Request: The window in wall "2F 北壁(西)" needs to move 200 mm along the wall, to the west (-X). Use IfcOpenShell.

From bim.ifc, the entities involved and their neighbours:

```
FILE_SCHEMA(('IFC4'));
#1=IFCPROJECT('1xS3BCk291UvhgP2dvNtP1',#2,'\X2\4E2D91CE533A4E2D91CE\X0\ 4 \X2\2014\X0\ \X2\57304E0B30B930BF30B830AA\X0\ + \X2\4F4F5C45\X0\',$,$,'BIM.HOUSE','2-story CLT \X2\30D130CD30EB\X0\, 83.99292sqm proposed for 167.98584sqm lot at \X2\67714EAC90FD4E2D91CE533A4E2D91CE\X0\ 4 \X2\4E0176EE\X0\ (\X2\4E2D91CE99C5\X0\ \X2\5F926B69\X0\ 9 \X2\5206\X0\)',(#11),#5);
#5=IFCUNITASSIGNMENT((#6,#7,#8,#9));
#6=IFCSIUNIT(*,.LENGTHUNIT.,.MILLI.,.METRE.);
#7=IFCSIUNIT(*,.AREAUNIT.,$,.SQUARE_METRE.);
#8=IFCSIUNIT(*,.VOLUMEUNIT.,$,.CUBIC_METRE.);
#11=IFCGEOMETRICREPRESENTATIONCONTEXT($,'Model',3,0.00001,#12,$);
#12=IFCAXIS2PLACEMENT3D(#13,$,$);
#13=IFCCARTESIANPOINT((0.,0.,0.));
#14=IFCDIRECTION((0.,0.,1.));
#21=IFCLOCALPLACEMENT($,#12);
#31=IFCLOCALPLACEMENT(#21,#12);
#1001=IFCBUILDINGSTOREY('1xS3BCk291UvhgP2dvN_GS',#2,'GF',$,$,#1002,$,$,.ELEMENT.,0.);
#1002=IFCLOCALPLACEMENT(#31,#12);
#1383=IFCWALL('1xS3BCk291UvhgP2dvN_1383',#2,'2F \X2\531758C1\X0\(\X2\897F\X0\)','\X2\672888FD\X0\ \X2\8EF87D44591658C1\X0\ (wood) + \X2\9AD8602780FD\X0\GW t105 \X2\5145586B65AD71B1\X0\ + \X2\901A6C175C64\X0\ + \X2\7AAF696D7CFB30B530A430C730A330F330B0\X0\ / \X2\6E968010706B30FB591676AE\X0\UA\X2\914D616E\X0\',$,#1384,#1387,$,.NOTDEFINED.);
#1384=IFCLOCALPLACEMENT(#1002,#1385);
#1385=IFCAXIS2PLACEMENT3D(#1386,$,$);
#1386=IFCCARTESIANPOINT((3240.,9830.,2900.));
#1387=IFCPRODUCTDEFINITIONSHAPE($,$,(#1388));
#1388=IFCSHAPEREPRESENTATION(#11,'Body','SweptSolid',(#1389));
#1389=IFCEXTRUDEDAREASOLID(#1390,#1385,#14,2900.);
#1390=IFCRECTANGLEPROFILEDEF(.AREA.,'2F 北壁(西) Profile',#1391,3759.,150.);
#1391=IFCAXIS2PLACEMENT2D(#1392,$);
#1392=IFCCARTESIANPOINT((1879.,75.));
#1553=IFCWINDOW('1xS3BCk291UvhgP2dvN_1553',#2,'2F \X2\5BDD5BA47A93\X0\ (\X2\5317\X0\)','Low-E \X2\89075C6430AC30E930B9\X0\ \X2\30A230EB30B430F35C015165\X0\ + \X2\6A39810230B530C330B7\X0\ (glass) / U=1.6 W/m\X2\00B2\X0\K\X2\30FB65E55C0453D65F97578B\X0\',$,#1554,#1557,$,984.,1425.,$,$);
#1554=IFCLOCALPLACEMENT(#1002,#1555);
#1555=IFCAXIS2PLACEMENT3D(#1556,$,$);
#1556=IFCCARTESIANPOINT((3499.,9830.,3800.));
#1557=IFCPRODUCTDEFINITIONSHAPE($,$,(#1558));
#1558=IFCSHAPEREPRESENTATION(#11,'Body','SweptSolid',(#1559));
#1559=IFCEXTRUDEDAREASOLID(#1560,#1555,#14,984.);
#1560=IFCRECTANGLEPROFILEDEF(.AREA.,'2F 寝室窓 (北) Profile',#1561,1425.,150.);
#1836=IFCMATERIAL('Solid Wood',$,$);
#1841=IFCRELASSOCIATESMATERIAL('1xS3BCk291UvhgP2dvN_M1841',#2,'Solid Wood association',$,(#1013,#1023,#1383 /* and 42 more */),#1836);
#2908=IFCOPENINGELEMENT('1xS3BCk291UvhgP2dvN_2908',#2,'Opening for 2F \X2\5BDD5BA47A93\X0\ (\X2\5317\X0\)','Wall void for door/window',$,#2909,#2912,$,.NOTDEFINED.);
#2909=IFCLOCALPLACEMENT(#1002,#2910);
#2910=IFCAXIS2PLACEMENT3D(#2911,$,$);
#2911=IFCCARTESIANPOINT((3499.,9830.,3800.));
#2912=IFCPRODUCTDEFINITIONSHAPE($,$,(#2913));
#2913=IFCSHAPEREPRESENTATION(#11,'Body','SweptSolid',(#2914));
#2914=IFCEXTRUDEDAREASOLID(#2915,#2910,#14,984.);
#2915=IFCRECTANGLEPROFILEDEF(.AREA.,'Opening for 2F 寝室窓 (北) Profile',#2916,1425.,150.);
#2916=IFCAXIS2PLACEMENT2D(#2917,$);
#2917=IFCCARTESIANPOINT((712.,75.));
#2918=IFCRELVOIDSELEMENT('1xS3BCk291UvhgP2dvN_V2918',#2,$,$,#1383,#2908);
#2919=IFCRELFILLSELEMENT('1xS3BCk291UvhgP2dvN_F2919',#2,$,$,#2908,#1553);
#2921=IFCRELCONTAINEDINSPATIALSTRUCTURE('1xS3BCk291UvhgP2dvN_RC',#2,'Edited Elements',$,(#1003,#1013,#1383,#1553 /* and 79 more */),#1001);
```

```python
import ifcopenshell
import ifcopenshell.api.geometry
import ifcopenshell.util.placement
import ifcopenshell.util.unit

model = ifcopenshell.open("bim.ifc")
unit_scale = ifcopenshell.util.unit.calculate_unit_scale(model)

window = model.by_guid("1xS3BCk291UvhgP2dvN_1553")
opening = window.FillsVoids[0].RelatingOpeningElement
wall = opening.VoidsElements[0].RelatingBuildingElement

wall_matrix = ifcopenshell.util.placement.get_local_placement(wall.ObjectPlacement)
shift = wall_matrix[:3, 0] * -0.2 / unit_scale
before = ifcopenshell.util.placement.get_local_placement(window.ObjectPlacement)[:3, 3].copy()

# The window is not placed relative to its opening, so move both.
for product in (opening, window):
    matrix = ifcopenshell.util.placement.get_local_placement(product.ObjectPlacement)
    matrix[:3, 3] += shift
    ifcopenshell.api.geometry.edit_object_placement(model, product=product, matrix=matrix, is_si=False)

after = ifcopenshell.util.placement.get_local_placement(window.ObjectPlacement)[:3, 3]
print("window moved by", (after - before).round(3) + 0.0)

model.write("bim-out.ifc")
```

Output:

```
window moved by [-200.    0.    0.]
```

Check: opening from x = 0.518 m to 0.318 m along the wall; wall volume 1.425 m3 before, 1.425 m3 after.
